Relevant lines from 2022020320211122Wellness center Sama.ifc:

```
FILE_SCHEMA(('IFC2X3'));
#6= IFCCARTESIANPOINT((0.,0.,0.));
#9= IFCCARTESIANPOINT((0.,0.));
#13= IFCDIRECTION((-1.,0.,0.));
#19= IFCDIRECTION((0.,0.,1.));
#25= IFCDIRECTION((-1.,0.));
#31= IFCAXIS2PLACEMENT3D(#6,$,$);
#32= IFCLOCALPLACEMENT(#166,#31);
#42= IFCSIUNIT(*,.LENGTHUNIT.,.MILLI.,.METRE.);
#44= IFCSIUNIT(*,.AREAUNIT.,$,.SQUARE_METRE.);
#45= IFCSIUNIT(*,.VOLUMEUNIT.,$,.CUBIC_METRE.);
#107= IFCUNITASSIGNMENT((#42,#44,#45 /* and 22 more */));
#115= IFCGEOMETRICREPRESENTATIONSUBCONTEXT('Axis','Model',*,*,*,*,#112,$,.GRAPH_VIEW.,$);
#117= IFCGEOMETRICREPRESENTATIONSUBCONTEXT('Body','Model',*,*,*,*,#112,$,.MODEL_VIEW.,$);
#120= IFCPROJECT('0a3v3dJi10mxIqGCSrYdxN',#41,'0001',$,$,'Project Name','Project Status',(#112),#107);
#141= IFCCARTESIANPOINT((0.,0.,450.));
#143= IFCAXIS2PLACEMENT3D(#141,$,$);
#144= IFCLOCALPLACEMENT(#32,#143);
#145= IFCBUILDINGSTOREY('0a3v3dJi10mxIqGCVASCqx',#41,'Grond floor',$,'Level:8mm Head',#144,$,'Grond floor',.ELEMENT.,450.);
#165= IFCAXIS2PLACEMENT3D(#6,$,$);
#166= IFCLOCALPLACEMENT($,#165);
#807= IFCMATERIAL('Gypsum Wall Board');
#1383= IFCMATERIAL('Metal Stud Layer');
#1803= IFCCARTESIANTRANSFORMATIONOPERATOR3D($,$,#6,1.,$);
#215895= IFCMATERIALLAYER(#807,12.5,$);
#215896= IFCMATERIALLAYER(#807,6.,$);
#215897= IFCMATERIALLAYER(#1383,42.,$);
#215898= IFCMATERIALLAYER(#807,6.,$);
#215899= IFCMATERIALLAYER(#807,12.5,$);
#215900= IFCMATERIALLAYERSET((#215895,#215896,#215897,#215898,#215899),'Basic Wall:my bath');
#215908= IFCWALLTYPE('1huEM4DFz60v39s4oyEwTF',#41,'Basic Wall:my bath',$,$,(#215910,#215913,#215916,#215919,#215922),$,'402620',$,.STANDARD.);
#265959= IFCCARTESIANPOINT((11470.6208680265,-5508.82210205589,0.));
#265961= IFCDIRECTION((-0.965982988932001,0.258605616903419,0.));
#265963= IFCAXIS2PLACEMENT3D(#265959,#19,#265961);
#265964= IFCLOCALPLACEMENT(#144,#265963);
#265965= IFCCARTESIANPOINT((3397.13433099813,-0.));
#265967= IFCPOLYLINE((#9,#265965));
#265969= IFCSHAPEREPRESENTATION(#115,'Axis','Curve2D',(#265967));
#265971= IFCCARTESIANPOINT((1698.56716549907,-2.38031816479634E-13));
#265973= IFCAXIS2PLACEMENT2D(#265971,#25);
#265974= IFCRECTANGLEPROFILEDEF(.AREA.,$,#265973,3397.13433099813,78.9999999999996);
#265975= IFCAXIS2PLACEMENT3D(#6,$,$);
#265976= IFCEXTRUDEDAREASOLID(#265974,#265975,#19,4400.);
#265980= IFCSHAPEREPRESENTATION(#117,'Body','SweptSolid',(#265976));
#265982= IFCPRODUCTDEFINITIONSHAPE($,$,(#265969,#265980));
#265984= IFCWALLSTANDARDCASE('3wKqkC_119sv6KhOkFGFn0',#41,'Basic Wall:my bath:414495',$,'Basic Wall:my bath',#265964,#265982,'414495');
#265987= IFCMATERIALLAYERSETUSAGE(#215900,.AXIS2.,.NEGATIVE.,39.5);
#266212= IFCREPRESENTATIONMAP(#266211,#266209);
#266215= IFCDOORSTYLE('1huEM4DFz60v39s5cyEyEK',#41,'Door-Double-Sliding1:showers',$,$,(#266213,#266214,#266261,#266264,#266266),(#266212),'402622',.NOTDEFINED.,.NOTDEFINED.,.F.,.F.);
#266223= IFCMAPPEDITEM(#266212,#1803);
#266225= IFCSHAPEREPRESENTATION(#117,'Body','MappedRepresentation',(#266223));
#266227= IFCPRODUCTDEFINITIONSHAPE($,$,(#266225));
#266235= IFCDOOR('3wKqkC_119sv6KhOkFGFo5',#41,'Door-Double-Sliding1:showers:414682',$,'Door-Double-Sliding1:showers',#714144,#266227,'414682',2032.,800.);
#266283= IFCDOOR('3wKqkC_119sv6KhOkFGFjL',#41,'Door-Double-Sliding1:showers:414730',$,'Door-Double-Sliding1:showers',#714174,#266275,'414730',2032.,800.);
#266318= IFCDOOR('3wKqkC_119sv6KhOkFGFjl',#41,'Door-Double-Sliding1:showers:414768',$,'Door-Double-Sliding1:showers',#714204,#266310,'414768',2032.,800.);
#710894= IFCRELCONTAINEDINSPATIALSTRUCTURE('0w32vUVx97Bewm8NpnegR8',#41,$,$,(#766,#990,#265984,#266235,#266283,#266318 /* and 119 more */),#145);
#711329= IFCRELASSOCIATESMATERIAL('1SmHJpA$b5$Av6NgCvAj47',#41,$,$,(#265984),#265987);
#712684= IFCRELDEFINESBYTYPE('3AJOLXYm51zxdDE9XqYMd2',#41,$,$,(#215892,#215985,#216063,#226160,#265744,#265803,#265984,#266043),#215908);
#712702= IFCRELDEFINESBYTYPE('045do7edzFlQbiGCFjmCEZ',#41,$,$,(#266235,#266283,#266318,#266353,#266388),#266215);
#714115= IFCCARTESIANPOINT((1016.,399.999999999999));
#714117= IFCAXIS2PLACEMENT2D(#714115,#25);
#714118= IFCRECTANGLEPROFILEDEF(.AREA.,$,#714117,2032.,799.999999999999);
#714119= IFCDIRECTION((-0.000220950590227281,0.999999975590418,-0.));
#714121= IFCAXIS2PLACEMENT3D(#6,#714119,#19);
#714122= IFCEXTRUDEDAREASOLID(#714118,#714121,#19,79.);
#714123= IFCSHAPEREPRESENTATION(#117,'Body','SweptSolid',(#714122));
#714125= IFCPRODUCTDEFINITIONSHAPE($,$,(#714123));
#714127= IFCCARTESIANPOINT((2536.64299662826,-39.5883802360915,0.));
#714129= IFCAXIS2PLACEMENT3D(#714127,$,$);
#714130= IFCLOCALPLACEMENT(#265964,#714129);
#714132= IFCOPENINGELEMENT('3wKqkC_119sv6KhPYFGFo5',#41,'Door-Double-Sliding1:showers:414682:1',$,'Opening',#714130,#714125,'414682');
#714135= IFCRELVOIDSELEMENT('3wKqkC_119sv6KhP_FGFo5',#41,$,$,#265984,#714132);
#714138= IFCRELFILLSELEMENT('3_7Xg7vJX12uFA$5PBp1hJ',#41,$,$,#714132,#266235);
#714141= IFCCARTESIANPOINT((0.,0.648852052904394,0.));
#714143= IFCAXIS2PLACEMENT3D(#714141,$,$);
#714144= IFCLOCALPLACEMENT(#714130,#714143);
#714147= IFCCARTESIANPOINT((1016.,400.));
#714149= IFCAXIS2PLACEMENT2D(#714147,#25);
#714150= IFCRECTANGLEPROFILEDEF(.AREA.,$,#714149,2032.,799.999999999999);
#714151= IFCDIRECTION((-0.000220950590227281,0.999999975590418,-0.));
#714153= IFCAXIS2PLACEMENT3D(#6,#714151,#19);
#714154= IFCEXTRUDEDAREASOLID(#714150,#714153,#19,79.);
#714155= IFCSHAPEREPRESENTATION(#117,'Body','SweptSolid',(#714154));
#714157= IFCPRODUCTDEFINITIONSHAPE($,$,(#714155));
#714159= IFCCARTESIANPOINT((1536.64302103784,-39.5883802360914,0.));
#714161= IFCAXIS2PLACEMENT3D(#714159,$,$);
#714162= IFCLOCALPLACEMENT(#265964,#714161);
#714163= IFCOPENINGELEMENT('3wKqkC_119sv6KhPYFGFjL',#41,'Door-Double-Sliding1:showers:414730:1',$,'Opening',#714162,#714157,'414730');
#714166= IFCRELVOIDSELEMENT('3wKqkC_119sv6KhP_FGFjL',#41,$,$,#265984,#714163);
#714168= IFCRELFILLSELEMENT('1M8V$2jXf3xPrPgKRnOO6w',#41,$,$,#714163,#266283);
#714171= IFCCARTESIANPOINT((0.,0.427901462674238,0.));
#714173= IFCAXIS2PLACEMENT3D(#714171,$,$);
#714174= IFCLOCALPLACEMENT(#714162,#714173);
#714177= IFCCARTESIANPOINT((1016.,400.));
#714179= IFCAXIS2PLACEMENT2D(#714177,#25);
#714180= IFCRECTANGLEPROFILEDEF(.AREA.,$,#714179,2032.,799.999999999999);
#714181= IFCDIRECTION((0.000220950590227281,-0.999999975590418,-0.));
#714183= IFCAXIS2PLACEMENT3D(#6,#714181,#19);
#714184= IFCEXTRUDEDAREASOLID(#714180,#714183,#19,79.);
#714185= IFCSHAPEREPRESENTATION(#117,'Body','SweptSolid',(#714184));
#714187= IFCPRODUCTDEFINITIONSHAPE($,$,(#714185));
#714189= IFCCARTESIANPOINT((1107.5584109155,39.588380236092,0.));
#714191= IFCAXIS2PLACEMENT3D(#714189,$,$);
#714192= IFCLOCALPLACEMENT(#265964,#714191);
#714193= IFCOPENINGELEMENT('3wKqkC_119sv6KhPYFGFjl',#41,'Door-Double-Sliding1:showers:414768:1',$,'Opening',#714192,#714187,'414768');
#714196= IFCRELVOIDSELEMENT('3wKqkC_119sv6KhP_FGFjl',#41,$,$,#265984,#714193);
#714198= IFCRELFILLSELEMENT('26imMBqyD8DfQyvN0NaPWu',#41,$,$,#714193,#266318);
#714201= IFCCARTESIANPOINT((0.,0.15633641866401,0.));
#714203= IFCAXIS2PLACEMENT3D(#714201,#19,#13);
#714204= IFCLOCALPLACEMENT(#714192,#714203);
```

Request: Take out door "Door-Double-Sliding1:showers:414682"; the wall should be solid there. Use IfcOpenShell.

```python
import ifcopenshell
import ifcopenshell.api.feature
import ifcopenshell.api.root
import ifcopenshell.geom
import ifcopenshell.util.shape

model = ifcopenshell.open("2022020320211122Wellness center Sama.ifc")
settings = ifcopenshell.geom.settings()


def volume(element):
    """Net volume in cubic metres, openings subtracted."""
    shape = ifcopenshell.geom.create_shape(settings, element)
    return ifcopenshell.util.shape.get_volume(shape.geometry)


door = model.by_id(266235)
opening = door.FillsVoids[0].RelatingOpeningElement
wall = opening.VoidsElements[0].RelatingBuildingElement
before = volume(wall)

ifcopenshell.api.root.remove_product(model, product=door)
ifcopenshell.api.feature.remove_feature(model, feature=opening)

after = volume(wall)

print(f"wall volume {before:.3f} -> {after:.3f} m3")

model.write("2022020320211122Wellness center Sama-out.ifc")
```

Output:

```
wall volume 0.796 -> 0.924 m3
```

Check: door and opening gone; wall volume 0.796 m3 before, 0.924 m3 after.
